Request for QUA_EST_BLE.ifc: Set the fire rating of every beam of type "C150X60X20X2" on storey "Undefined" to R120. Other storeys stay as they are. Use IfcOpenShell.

First a look at what the model holds.

```python
import ifcopenshell
import ifcopenshell.util.element

model = ifcopenshell.open("QUA_EST_BLE.ifc")
print(model.schema)
storey = next(s for s in model.by_type("IfcBuildingStorey") if s.Name == "Undefined")
beams = [e for e in ifcopenshell.util.element.get_decomposition(storey) if e.is_a("IfcBeam")]
seen = {}
for e in beams:
    element_type = ifcopenshell.util.element.get_type(e)
    key = (element_type.Name if element_type != e and element_type else None, ifcopenshell.util.element.get_pset(e, "Pset_BeamCommon", "FireRating"))
    seen[key] = seen.get(key, 0) + 1
for (name, value), count in sorted(seen.items(), key=str):
    print(count, "x", name, "|", value)
```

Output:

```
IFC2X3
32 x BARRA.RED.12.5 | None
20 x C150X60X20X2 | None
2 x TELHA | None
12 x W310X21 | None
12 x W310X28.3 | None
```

```python
import ifcopenshell
import ifcopenshell.api.pset
import ifcopenshell.util.element

model = ifcopenshell.open("QUA_EST_BLE.ifc")

storey = next(s for s in model.by_type("IfcBuildingStorey") if s.Name == "Undefined")
beams = [e for e in ifcopenshell.util.element.get_decomposition(storey) if e.is_a("IfcBeam")]

count = 0
for e in beams:
    element_type = ifcopenshell.util.element.get_type(e)
    if element_type in (None, e) or element_type.Name != "C150X60X20X2":
        continue
    found = ifcopenshell.util.element.get_pset(e, "Pset_BeamCommon", should_inherit=False)
    if found:
        pset = model.by_id(found["id"])
        if len(ifcopenshell.util.element.get_elements_by_pset(pset)) > 1:
            pset = ifcopenshell.api.pset.unshare_pset(model, products=[e], pset=pset)[0]
    else:
        pset = ifcopenshell.api.pset.add_pset(model, product=e, name="Pset_BeamCommon")
    ifcopenshell.api.pset.edit_pset(model, pset=pset, properties={"FireRating": "R120"})
    count += 1

print(count, "beams updated")

model.write("QUA_EST_BLE_updated.ifc")
```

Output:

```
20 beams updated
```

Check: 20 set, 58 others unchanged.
